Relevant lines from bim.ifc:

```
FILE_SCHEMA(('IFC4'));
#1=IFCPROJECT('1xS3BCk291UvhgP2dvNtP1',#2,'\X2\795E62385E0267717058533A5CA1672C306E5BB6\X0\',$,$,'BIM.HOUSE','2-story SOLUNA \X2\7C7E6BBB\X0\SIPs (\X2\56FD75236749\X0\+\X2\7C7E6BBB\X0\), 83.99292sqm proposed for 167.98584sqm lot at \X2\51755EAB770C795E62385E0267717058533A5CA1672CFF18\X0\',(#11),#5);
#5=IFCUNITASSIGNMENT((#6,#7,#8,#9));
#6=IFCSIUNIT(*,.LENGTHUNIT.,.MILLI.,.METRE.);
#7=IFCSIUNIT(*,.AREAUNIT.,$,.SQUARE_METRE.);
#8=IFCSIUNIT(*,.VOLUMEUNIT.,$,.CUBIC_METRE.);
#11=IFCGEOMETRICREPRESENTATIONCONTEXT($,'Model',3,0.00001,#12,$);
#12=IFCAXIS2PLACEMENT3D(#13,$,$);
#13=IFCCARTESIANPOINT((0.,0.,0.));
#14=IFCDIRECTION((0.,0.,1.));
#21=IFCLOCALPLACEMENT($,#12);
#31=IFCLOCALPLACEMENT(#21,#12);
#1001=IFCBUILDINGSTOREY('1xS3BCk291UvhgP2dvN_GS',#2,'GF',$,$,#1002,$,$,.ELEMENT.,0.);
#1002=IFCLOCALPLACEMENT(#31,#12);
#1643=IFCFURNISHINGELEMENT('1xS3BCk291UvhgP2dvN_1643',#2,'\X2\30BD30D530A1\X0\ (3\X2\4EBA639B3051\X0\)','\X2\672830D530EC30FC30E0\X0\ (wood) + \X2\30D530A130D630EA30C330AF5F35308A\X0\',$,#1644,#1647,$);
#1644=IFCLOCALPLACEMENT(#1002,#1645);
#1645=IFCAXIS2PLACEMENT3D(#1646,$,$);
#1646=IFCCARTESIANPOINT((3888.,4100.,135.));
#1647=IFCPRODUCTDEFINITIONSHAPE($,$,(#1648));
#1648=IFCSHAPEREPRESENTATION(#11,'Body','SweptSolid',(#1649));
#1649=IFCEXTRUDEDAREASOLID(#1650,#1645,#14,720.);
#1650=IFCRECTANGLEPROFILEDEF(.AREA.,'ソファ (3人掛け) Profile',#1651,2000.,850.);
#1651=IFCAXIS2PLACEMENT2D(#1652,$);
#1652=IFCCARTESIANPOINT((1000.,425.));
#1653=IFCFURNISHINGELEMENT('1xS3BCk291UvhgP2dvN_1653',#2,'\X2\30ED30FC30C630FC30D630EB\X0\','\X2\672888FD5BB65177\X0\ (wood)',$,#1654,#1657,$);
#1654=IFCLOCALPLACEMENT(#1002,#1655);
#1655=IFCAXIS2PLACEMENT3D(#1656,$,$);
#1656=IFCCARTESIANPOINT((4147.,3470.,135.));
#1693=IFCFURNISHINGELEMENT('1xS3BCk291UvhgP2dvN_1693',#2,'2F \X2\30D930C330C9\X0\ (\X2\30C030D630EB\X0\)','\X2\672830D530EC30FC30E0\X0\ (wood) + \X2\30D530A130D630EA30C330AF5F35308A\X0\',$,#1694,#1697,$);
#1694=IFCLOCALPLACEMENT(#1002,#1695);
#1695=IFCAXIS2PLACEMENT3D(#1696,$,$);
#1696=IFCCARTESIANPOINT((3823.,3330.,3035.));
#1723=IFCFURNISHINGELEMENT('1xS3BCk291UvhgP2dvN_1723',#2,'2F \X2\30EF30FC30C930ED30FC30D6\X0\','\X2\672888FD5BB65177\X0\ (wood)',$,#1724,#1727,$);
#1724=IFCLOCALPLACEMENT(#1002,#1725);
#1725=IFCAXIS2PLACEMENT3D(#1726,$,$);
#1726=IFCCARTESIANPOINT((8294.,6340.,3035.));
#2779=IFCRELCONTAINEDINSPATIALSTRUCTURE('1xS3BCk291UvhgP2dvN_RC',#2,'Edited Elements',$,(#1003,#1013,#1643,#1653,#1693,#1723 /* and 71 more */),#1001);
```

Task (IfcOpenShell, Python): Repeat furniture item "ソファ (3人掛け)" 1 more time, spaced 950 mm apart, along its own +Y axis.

```python
import ifcopenshell
import ifcopenshell.api.geometry
import ifcopenshell.api.root
import ifcopenshell.util.element
import ifcopenshell.util.placement
import ifcopenshell.util.unit

model = ifcopenshell.open("bim.ifc")
unit_scale = ifcopenshell.util.unit.calculate_unit_scale(model)


def reuse_history(source, copy):
    """copy_class also copies each property set's owner history, people and application; keep the originals."""
    for rel in copy.IsDefinedBy:
        if rel.is_a("IfcRelDefinesByProperties") and (history := rel.RelatingPropertyDefinition.OwnerHistory):
            rel.RelatingPropertyDefinition.OwnerHistory = source.OwnerHistory
            ifcopenshell.util.element.remove_deep2(model, history)


source = model.by_guid("1xS3BCk291UvhgP2dvN_1643")
base = ifcopenshell.util.placement.get_local_placement(source.ObjectPlacement)
step = base[:3, 1] * 0.95 / unit_scale

for i in range(1, 2):
    copy = ifcopenshell.api.root.copy_class(model, product=source)
    copy.Representation = ifcopenshell.util.element.copy_deep(
        model, source.Representation, exclude=["IfcGeometricRepresentationContext", "IfcRepresentationMap"]
    )
    reuse_history(source, copy)
    matrix = base.copy()
    matrix[:3, 3] += i * step
    print("added at", matrix[:3, 3].round(3) + 0.0)
    ifcopenshell.api.geometry.edit_object_placement(model, product=copy, matrix=matrix, is_si=False)

model.write("bim_v2.ifc")
```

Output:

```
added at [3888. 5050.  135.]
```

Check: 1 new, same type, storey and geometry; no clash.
